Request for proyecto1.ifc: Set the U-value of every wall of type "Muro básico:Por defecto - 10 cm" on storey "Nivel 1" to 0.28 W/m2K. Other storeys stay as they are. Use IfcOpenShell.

First a look at what the model holds.

```python
import ifcopenshell
import ifcopenshell.util.element

model = ifcopenshell.open("proyecto1.ifc")
print(model.schema)
storey = next(s for s in model.by_type("IfcBuildingStorey") if s.Name == "Nivel 1")
walls = [e for e in ifcopenshell.util.element.get_decomposition(storey) if e.is_a("IfcWall")]
seen = {}
for e in walls:
    element_type = ifcopenshell.util.element.get_type(e)
    key = (element_type.Name if element_type != e and element_type else None, ifcopenshell.util.element.get_pset(e, "Pset_WallCommon", "ThermalTransmittance"))
    seen[key] = seen.get(key, 0) + 1
for (name, value), count in sorted(seen.items(), key=str):
    print(count, "x", name, "|", value)
```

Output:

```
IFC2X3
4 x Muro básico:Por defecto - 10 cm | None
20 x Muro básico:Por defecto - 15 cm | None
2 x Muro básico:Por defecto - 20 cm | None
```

```python
import ifcopenshell
import ifcopenshell.api.pset
import ifcopenshell.util.element

model = ifcopenshell.open("proyecto1.ifc")

storey = next(s for s in model.by_type("IfcBuildingStorey") if s.Name == "Nivel 1")
walls = [e for e in ifcopenshell.util.element.get_decomposition(storey) if e.is_a("IfcWall")]

count = 0
for e in walls:
    element_type = ifcopenshell.util.element.get_type(e)
    if element_type in (None, e) or element_type.Name != "Muro básico:Por defecto - 10 cm":
        continue
    # add_pset returns the element's existing set when there is one.
    pset = ifcopenshell.api.pset.add_pset(model, product=e, name="Pset_WallCommon")
    ifcopenshell.api.pset.edit_pset(model, pset=pset, properties={"ThermalTransmittance": 0.28})
    count += 1

print(count, "walls updated")

model.write("proyecto1_edited.ifc")
```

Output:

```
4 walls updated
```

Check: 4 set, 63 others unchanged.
